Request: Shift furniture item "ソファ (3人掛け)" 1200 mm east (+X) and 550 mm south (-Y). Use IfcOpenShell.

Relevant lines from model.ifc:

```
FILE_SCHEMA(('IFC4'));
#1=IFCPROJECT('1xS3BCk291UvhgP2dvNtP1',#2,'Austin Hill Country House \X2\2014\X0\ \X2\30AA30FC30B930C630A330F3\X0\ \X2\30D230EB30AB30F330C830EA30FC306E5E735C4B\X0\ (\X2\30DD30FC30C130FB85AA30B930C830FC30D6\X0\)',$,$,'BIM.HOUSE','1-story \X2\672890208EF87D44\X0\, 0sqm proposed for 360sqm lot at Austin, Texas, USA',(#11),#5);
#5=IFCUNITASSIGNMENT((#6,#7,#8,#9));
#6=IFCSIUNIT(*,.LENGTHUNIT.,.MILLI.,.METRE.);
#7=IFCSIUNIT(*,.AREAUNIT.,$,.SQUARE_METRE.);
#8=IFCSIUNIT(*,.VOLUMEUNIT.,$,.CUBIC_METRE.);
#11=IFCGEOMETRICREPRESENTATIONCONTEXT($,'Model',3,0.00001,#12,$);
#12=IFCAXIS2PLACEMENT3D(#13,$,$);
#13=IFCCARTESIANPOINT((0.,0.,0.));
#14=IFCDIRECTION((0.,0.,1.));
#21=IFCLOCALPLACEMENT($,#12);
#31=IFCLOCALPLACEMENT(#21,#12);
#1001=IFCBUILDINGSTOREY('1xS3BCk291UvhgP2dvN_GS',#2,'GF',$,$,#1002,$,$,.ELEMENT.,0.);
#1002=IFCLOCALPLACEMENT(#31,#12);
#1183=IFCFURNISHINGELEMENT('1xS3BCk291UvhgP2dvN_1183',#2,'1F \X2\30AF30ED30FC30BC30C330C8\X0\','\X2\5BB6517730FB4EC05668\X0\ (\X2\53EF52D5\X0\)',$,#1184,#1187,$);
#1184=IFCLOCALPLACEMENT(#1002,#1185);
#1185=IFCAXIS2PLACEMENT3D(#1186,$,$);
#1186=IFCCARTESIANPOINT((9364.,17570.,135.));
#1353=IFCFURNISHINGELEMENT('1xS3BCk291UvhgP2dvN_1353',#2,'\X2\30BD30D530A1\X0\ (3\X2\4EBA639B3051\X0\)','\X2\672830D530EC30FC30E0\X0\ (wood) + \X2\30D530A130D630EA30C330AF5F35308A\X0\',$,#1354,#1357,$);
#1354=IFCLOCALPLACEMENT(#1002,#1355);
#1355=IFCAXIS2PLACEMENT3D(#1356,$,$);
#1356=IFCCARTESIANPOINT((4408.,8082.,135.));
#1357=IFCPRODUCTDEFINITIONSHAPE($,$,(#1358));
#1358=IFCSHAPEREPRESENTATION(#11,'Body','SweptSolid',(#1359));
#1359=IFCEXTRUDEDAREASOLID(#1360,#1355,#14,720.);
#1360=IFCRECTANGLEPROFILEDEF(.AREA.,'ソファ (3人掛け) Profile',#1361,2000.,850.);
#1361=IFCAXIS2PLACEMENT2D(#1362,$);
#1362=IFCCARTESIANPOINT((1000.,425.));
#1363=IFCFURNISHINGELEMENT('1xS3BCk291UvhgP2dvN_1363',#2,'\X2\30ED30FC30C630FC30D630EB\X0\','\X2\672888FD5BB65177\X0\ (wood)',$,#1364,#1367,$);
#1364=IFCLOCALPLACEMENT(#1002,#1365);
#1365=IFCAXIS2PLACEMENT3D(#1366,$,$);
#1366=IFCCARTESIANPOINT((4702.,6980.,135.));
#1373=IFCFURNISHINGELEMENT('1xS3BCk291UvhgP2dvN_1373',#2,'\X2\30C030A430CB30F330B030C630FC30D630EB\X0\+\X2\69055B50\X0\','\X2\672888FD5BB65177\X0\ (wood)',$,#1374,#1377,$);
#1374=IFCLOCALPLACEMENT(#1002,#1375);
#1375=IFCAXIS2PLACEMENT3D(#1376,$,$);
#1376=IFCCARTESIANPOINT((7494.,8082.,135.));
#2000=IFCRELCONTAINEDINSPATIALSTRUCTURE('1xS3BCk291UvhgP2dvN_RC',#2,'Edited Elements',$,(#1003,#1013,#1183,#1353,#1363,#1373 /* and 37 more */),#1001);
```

```python
import ifcopenshell
import ifcopenshell.api.geometry
import ifcopenshell.util.placement
import ifcopenshell.util.unit

model = ifcopenshell.open("model.ifc")
unit_scale = ifcopenshell.util.unit.calculate_unit_scale(model)

item = model.by_guid("1xS3BCk291UvhgP2dvN_1353")
matrix = ifcopenshell.util.placement.get_local_placement(item.ObjectPlacement)
matrix[0, 3] += 1.2 / unit_scale
matrix[1, 3] -= 0.55 / unit_scale
ifcopenshell.api.geometry.edit_object_placement(model, product=item, matrix=matrix, is_si=False)

print(ifcopenshell.util.placement.get_local_placement(item.ObjectPlacement).round(3) + 0.0)

model.write("model_v2.ifc")
```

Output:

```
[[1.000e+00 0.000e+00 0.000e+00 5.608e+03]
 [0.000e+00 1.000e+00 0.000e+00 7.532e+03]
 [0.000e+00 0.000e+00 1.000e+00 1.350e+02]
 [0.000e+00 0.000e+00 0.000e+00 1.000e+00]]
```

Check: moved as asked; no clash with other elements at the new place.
